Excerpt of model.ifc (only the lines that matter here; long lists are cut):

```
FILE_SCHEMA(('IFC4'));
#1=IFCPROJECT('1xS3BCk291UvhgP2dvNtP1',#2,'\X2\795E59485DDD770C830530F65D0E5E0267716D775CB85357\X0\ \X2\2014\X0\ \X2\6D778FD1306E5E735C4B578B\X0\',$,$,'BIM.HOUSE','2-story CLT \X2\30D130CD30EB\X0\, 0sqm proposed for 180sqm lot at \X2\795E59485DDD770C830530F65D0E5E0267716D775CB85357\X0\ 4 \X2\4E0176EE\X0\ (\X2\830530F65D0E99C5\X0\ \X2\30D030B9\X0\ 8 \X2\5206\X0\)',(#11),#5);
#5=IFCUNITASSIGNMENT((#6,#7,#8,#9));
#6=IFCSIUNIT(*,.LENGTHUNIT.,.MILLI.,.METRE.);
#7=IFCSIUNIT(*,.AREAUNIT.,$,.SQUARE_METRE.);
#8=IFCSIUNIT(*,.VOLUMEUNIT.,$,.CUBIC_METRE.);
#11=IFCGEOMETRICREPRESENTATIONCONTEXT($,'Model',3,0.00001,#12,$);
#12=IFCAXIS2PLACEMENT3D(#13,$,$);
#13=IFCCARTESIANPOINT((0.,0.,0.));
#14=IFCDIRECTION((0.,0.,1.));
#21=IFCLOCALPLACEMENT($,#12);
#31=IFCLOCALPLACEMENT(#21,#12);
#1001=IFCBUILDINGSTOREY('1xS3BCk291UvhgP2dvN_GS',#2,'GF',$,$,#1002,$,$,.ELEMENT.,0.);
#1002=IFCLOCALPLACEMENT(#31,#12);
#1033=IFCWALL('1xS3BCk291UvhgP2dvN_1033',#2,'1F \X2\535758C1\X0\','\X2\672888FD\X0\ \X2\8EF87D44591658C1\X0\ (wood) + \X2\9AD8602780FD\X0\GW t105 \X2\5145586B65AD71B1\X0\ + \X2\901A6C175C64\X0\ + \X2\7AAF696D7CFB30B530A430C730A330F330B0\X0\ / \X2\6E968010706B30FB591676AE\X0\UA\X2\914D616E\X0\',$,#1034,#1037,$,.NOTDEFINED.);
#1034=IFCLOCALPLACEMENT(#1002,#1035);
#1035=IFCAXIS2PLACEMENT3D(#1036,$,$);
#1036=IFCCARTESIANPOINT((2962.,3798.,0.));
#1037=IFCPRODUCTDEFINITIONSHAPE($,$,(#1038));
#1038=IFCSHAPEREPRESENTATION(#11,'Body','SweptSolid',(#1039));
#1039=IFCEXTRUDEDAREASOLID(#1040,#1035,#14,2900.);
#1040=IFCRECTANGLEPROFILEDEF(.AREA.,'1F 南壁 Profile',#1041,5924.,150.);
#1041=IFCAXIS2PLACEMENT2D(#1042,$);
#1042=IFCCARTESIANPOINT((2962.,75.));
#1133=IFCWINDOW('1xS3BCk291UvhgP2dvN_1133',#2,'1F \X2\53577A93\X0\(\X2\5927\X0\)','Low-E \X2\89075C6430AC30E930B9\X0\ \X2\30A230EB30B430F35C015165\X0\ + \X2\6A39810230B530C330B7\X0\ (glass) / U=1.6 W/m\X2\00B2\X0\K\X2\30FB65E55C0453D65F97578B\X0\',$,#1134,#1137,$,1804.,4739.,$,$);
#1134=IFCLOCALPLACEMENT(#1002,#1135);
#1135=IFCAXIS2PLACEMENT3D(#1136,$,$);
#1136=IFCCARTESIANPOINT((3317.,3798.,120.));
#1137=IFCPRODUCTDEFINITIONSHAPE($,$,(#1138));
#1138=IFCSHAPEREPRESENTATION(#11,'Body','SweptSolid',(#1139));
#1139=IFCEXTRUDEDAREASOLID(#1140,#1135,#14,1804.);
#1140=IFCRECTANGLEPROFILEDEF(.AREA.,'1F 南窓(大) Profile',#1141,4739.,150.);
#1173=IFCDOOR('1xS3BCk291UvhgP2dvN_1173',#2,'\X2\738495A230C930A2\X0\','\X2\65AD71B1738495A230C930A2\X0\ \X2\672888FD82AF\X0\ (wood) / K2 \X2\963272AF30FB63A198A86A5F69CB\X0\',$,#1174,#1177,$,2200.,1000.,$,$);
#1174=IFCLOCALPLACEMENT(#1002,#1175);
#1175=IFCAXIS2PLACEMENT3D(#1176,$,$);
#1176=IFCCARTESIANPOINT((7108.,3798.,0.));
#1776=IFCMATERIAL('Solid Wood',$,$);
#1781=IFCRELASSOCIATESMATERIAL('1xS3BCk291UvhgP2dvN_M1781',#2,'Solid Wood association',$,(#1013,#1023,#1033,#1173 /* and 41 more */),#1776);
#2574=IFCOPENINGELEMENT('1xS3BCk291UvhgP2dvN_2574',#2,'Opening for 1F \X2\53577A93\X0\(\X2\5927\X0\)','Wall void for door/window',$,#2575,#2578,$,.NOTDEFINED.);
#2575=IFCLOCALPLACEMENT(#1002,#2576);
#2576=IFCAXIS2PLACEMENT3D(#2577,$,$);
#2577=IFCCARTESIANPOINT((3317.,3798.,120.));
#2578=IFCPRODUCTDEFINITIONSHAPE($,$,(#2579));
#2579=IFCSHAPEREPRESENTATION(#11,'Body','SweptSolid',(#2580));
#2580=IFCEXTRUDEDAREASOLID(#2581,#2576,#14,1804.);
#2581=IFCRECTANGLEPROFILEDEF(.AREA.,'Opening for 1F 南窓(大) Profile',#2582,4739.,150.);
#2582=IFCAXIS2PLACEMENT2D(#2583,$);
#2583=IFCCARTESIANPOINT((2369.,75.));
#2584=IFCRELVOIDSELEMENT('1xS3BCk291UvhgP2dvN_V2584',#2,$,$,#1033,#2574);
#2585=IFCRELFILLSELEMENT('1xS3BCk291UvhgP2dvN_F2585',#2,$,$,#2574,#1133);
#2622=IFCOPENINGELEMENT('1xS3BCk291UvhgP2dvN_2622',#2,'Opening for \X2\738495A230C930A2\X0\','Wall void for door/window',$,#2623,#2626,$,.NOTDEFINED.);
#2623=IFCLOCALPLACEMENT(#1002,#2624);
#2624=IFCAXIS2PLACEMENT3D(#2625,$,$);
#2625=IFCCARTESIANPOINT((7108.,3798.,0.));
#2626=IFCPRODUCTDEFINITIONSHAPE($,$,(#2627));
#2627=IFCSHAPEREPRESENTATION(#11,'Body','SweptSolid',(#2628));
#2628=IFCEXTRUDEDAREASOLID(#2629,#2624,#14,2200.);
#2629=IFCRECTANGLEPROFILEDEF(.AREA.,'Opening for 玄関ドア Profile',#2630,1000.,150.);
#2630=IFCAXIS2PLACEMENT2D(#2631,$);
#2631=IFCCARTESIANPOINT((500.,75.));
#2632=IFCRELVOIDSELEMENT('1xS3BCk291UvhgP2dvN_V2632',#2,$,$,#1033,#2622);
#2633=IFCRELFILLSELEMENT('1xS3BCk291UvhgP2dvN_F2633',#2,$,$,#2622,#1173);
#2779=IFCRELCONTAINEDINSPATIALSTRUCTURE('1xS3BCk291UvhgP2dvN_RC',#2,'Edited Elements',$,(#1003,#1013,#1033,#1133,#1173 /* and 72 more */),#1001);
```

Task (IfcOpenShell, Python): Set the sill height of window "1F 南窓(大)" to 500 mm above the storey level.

```python
import numpy as np
import ifcopenshell
import ifcopenshell.api.geometry
import ifcopenshell.geom
import ifcopenshell.util.element
import ifcopenshell.util.placement
import ifcopenshell.util.shape
import ifcopenshell.util.unit

model = ifcopenshell.open("model.ifc")
unit_scale = ifcopenshell.util.unit.calculate_unit_scale(model)

window = model.by_guid("1xS3BCk291UvhgP2dvN_1133")
opening = window.FillsVoids[0].RelatingOpeningElement
storey = ifcopenshell.util.element.get_container(window, ifc_class="IfcBuildingStorey")
level = ifcopenshell.util.placement.get_local_placement(storey.ObjectPlacement)[2, 3]

# The opening's origin need not be at the sill, so measure its lowest point.
shape = ifcopenshell.geom.create_shape(ifcopenshell.geom.settings(), opening)
bottom = ifcopenshell.util.shape.get_shape_bottom_elevation(shape, shape.geometry) / unit_scale
dz = level + 0.5 / unit_scale - bottom

shift = np.array([0.0, 0.0, dz])
# The window is not placed relative to its opening, so move both.
for product in (opening, window):
    matrix = ifcopenshell.util.placement.get_local_placement(product.ObjectPlacement)
    matrix[:3, 3] += shift
    ifcopenshell.api.geometry.edit_object_placement(model, product=product, matrix=matrix, is_si=False)

print(f"moved by {dz * unit_scale:+.3f} m")

model.write("model_edited.ifc")
```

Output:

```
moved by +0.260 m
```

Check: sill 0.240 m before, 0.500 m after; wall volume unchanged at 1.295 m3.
